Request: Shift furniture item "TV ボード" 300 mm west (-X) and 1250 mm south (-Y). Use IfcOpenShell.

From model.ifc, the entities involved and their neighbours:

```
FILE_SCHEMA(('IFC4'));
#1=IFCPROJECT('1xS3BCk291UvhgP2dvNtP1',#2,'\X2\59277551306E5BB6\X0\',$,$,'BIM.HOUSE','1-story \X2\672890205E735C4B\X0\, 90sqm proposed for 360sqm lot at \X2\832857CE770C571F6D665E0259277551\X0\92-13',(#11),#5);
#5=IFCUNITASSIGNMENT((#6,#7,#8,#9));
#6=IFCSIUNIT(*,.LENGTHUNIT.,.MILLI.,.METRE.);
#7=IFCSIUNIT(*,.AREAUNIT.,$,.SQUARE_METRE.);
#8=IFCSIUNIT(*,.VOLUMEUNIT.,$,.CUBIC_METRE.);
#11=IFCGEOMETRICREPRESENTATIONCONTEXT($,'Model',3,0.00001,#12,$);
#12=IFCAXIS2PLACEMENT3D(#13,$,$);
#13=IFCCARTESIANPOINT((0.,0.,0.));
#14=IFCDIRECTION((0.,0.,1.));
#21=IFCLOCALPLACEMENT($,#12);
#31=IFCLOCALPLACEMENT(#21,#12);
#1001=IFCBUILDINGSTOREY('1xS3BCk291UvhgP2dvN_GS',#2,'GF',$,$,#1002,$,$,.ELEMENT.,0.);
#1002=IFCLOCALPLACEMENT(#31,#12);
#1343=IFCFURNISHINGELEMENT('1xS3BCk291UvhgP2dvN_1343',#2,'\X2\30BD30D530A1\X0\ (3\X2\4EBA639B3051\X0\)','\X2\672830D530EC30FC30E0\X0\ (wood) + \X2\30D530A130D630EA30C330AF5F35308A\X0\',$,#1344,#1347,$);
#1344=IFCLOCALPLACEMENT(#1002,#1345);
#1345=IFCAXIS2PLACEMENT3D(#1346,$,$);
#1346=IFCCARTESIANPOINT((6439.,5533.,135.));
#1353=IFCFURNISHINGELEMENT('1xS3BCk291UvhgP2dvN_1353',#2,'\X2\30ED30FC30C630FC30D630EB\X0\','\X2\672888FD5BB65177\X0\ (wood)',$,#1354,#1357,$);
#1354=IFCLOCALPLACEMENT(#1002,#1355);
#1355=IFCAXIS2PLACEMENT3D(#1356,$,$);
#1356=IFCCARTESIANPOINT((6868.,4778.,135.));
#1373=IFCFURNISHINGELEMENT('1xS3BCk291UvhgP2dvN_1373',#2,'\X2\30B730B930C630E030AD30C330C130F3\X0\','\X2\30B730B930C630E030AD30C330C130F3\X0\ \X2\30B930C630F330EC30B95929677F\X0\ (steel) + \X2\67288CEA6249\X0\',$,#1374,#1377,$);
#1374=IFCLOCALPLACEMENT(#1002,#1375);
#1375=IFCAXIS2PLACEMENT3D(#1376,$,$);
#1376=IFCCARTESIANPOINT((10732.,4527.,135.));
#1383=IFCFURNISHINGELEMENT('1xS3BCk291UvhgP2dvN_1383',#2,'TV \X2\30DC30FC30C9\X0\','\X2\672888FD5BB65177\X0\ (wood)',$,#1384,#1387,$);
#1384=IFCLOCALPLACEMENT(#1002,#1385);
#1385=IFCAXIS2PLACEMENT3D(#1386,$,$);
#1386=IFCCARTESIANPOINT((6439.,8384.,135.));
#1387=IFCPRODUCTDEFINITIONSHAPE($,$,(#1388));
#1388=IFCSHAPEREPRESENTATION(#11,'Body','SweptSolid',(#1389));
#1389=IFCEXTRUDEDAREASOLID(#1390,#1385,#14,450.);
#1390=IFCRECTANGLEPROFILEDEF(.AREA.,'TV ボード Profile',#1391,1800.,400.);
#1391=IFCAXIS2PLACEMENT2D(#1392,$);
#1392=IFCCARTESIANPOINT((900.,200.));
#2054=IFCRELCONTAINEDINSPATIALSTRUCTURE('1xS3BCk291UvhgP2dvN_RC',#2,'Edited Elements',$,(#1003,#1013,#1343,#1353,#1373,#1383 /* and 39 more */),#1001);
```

```python
import ifcopenshell
import ifcopenshell.api.geometry
import ifcopenshell.util.placement
import ifcopenshell.util.unit

model = ifcopenshell.open("model.ifc")
unit_scale = ifcopenshell.util.unit.calculate_unit_scale(model)

item = model.by_guid("1xS3BCk291UvhgP2dvN_1383")
matrix = ifcopenshell.util.placement.get_local_placement(item.ObjectPlacement)
matrix[0, 3] -= 0.3 / unit_scale
matrix[1, 3] -= 1.25 / unit_scale
ifcopenshell.api.geometry.edit_object_placement(model, product=item, matrix=matrix, is_si=False)

print(ifcopenshell.util.placement.get_local_placement(item.ObjectPlacement).round(3) + 0.0)

model.write("model-out.ifc")
```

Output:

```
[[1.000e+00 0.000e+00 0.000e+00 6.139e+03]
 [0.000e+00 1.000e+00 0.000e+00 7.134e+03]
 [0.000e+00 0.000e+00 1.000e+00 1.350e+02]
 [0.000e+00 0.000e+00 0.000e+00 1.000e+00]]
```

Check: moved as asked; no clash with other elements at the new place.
